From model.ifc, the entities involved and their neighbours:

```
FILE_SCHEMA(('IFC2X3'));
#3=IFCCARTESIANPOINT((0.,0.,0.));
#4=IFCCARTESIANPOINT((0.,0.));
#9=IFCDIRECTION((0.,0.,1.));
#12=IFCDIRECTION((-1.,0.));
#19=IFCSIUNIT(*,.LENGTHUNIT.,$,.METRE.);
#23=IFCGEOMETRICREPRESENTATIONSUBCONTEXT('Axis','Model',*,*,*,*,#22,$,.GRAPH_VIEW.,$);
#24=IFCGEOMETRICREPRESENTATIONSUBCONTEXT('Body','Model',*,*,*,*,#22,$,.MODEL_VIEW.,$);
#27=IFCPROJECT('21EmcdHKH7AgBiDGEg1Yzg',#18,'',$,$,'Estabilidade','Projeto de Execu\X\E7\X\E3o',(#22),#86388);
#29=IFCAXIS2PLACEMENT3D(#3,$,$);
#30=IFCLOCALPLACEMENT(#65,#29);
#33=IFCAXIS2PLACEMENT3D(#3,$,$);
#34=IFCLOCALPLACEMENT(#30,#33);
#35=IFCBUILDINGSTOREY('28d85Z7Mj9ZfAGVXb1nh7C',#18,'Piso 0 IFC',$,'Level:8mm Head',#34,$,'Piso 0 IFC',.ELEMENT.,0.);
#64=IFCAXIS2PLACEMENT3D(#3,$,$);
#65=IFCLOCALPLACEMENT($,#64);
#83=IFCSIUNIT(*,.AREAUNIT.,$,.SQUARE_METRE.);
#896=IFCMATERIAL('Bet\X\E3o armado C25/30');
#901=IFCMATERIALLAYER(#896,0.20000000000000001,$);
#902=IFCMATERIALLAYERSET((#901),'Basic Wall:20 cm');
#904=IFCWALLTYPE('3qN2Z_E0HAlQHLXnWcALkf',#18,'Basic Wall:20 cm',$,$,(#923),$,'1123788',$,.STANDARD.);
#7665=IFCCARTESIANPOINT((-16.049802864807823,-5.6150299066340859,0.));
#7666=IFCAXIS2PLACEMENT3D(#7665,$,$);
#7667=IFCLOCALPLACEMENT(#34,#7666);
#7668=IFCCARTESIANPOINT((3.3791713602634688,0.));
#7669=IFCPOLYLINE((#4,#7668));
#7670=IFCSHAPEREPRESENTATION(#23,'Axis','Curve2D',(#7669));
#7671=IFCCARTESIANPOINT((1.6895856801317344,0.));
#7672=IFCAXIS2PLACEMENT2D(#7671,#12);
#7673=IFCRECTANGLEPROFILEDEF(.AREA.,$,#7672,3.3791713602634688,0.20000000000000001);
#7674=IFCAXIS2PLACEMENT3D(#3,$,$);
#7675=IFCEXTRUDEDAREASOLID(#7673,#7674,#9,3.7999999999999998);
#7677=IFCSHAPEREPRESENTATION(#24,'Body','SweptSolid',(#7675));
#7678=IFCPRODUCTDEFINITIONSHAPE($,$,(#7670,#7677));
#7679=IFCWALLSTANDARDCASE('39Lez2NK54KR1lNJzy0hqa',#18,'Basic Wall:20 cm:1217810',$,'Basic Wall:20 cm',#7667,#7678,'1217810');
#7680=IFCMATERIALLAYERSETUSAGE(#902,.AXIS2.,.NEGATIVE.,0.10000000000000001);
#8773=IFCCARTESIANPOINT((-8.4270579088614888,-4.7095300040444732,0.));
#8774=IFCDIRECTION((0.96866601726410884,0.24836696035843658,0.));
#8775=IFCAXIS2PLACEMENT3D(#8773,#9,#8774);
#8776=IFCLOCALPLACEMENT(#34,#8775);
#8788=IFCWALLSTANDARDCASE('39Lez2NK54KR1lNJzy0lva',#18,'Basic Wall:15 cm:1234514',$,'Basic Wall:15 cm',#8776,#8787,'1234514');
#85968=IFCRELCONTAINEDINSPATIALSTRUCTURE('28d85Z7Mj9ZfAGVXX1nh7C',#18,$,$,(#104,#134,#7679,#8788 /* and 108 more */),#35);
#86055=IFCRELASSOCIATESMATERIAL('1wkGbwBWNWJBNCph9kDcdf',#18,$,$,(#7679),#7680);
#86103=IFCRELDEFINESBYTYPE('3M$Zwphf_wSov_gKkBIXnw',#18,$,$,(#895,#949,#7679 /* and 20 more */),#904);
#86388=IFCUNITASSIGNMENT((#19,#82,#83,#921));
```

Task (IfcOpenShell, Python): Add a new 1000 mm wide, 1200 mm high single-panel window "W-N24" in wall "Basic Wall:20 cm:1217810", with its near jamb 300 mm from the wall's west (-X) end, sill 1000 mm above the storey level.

```python
import numpy as np
import ifcopenshell
import ifcopenshell.api.feature
import ifcopenshell.api.geometry
import ifcopenshell.api.root
import ifcopenshell.api.spatial
import ifcopenshell.api.type
import ifcopenshell.geom
import ifcopenshell.util.element
import ifcopenshell.util.placement
import ifcopenshell.util.representation
import ifcopenshell.util.shape
import ifcopenshell.util.unit

model = ifcopenshell.open("model.ifc")
unit_scale = ifcopenshell.util.unit.calculate_unit_scale(model)
settings = ifcopenshell.geom.settings()


def volume(element):
    """Net volume in cubic metres, openings subtracted."""
    shape = ifcopenshell.geom.create_shape(settings, element)
    return ifcopenshell.util.shape.get_volume(shape.geometry)


wall = model.by_guid("39Lez2NK54KR1lNJzy0hqa")
storey = ifcopenshell.util.element.get_container(wall, ifc_class="IfcBuildingStorey")
context = ifcopenshell.util.representation.get_context(model, "Model", "Body", "MODEL_VIEW")
before = volume(wall)

width, height, from_end, sill = 1, 1.2, 0.3, 1  # metres

# The wall runs along its own X axis, and the end named is its -X end.
wall_shape = ifcopenshell.geom.create_shape(settings, wall)
x, y, z = ifcopenshell.util.shape.get_vertices(wall_shape.geometry).T
start = x.min() + from_end
face, thickness = float(y.min()), float(y.max() - y.min())
wall_matrix = ifcopenshell.util.placement.get_local_placement(wall.ObjectPlacement)
level = ifcopenshell.util.placement.get_local_placement(storey.ObjectPlacement)[2, 3]


def in_wall(x, y):
    """Placement at x, y metres in the wall's axes, at sill height."""
    matrix = wall_matrix.copy()
    matrix[:, 3] = wall_matrix @ np.array([x / unit_scale, y / unit_scale, 0.0, 1.0])
    matrix[2, 3] = level + sill / unit_scale
    return matrix


# Opening: a box that overshoots both wall faces by 50 mm.
opening = ifcopenshell.api.root.create_entity(model, ifc_class="IfcOpeningElement")
box = ifcopenshell.api.geometry.add_wall_representation(
    model, context=context, length=width, height=height, thickness=thickness + 0.1
)
ifcopenshell.api.geometry.assign_representation(model, product=opening, representation=box)
ifcopenshell.api.geometry.edit_object_placement(model, product=opening, matrix=in_wall(start, face - 0.05), is_si=False)
ifcopenshell.api.feature.add_feature(model, feature=opening, element=wall)

window = ifcopenshell.api.root.create_entity(model, ifc_class="IfcWindow", name="W-N24")
window.OverallWidth, window.OverallHeight = width / unit_scale, height / unit_scale
body = ifcopenshell.api.geometry.add_window_representation(
    model,
    context=context,
    overall_width=window.OverallWidth,
    overall_height=window.OverallHeight,
    partition_type="SINGLE_PANEL",
)
ifcopenshell.api.geometry.assign_representation(model, product=window, representation=body)
ifcopenshell.api.spatial.assign_container(model, products=[window], relating_structure=storey)
fills = ifcopenshell.api.feature.add_filling(model, opening=opening, element=window)
fills.OwnerHistory = window.OwnerHistory  # required in IFC2X3

# IFC2X3 keeps the operation on the window style.
style = ifcopenshell.api.root.create_entity(model, ifc_class="IfcWindowStyle", name="W-N24")
style.OperationType, style.ConstructionType = "SINGLE_PANEL", "NOTDEFINED"
style.ParameterTakesPrecedence = style.Sizeable = False
ifcopenshell.api.type.assign_type(model, related_objects=[window], relating_type=style)

# Centre the window in the wall's thickness.
ifcopenshell.api.geometry.edit_object_placement(model, product=window, matrix=in_wall(start, face), is_si=False)
window_shape = ifcopenshell.geom.create_shape(settings, window)
depth = ifcopenshell.util.shape.get_vertices(window_shape.geometry)[:, 1]
offset = face + thickness / 2 - (depth.min() + depth.max()) / 2
ifcopenshell.api.geometry.edit_object_placement(model, product=window, matrix=in_wall(start, offset), is_si=False)

after = volume(wall)

print(f"wall volume {before:.3f} -> {after:.3f} m3")

model.write("model_rev.ifc")
```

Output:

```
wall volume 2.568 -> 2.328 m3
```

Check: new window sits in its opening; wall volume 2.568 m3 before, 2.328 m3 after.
